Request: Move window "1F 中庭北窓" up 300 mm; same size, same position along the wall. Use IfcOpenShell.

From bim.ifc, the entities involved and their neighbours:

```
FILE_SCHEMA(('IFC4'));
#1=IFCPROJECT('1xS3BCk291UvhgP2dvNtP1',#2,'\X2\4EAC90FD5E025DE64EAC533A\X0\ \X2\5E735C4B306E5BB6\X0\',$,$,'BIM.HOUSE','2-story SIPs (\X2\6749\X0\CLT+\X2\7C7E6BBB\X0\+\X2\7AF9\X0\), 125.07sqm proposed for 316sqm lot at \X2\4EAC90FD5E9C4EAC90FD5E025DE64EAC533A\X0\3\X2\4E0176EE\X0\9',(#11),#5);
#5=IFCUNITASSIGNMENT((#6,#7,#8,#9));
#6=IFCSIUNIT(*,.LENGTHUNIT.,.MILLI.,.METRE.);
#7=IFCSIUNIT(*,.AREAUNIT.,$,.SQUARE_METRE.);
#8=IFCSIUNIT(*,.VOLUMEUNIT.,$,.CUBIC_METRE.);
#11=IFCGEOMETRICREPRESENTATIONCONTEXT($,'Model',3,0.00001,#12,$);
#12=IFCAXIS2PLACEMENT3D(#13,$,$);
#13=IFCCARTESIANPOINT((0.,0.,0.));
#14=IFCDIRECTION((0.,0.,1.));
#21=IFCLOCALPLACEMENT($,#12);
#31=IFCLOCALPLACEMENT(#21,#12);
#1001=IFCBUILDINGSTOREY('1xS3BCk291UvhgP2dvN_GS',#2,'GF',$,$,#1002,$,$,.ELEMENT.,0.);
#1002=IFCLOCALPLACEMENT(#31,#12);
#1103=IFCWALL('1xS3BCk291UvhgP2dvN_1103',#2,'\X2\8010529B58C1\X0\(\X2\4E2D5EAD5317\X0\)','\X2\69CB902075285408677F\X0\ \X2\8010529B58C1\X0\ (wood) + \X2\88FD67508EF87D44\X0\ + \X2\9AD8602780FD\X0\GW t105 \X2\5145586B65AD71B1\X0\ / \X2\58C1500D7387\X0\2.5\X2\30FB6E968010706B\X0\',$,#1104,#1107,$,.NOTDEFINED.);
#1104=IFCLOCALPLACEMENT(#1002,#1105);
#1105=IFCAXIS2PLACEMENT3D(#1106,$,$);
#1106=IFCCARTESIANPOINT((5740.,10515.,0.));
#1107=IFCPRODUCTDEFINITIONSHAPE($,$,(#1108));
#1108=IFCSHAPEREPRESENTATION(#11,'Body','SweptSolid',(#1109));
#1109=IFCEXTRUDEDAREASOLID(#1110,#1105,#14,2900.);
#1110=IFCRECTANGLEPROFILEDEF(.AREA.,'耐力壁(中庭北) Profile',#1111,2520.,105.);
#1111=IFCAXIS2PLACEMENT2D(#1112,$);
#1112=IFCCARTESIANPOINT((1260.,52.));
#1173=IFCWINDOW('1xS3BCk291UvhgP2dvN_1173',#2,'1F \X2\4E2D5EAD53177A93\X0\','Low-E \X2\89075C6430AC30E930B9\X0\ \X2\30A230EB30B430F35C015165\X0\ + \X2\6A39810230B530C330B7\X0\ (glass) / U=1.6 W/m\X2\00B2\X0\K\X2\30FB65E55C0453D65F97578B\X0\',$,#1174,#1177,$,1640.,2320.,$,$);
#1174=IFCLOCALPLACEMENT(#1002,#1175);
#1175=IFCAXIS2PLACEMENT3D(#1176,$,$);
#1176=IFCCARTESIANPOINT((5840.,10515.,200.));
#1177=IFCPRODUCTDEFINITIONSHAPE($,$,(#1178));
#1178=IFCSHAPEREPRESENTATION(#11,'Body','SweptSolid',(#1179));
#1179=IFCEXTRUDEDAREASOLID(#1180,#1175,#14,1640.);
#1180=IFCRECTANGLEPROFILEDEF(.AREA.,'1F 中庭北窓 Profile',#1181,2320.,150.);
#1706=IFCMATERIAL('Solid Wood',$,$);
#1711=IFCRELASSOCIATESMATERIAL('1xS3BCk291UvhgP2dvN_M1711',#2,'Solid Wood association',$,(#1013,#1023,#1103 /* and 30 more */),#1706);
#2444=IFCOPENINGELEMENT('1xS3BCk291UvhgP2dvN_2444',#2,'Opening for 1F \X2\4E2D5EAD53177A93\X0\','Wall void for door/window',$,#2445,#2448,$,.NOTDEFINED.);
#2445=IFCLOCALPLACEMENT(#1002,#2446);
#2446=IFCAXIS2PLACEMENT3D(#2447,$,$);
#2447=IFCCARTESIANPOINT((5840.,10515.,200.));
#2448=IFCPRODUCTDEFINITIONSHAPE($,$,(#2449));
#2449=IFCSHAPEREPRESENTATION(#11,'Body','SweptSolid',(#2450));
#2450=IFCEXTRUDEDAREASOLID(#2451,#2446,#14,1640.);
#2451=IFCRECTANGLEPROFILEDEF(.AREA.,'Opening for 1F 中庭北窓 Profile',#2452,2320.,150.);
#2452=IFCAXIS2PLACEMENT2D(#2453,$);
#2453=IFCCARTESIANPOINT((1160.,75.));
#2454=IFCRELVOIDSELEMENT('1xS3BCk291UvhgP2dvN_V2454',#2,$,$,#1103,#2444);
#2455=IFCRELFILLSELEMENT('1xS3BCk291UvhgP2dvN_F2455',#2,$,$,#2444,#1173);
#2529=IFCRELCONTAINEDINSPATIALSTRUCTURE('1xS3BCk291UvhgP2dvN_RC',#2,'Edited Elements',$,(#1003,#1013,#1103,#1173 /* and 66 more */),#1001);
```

```python
import numpy as np
import ifcopenshell
import ifcopenshell.api.geometry
import ifcopenshell.util.placement
import ifcopenshell.util.unit

model = ifcopenshell.open("bim.ifc")
unit_scale = ifcopenshell.util.unit.calculate_unit_scale(model)

window = model.by_guid("1xS3BCk291UvhgP2dvN_1173")
opening = window.FillsVoids[0].RelatingOpeningElement
dz = 300.0

shift = np.array([0.0, 0.0, dz])
# The window is not placed relative to its opening, so move both.
for product in (opening, window):
    matrix = ifcopenshell.util.placement.get_local_placement(product.ObjectPlacement)
    matrix[:3, 3] += shift
    ifcopenshell.api.geometry.edit_object_placement(model, product=product, matrix=matrix, is_si=False)

print(f"moved by {dz * unit_scale:+.3f} m")

model.write("bim-out.ifc")
```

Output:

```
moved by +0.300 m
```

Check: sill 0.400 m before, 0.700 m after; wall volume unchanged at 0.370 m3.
